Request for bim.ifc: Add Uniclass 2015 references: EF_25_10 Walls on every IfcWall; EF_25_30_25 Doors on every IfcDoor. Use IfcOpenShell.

First a look at what the model holds.

```python
import ifcopenshell

model = ifcopenshell.open("bim.ifc")
print(model.schema)
print("classifications:", [c.Name for c in model.by_type("IfcClassification")])
for ifc_class in ("IfcDoor", "IfcRoof", "IfcStair", "IfcWall", "IfcWindow"):
    print(ifc_class, len(model.by_type(ifc_class)))
```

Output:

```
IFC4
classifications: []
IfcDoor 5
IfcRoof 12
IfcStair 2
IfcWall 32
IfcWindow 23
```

```python
import ifcopenshell
import ifcopenshell.api.classification

model = ifcopenshell.open("bim.ifc")

system = ifcopenshell.api.classification.add_classification(model, classification="Uniclass 2015")

codes = {
    "IfcWall": ("EF_25_10", "Walls"),
    "IfcDoor": ("EF_25_30_25", "Doors"),
}
for ifc_class, (code, name) in codes.items():
    products = model.by_type(ifc_class)
    ifcopenshell.api.classification.add_reference(
        model, products=products, classification=system, identification=code, name=name
    )
    print(code, len(products))

model.write("bim_v2.ifc")
```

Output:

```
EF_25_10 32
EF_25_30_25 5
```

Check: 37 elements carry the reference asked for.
